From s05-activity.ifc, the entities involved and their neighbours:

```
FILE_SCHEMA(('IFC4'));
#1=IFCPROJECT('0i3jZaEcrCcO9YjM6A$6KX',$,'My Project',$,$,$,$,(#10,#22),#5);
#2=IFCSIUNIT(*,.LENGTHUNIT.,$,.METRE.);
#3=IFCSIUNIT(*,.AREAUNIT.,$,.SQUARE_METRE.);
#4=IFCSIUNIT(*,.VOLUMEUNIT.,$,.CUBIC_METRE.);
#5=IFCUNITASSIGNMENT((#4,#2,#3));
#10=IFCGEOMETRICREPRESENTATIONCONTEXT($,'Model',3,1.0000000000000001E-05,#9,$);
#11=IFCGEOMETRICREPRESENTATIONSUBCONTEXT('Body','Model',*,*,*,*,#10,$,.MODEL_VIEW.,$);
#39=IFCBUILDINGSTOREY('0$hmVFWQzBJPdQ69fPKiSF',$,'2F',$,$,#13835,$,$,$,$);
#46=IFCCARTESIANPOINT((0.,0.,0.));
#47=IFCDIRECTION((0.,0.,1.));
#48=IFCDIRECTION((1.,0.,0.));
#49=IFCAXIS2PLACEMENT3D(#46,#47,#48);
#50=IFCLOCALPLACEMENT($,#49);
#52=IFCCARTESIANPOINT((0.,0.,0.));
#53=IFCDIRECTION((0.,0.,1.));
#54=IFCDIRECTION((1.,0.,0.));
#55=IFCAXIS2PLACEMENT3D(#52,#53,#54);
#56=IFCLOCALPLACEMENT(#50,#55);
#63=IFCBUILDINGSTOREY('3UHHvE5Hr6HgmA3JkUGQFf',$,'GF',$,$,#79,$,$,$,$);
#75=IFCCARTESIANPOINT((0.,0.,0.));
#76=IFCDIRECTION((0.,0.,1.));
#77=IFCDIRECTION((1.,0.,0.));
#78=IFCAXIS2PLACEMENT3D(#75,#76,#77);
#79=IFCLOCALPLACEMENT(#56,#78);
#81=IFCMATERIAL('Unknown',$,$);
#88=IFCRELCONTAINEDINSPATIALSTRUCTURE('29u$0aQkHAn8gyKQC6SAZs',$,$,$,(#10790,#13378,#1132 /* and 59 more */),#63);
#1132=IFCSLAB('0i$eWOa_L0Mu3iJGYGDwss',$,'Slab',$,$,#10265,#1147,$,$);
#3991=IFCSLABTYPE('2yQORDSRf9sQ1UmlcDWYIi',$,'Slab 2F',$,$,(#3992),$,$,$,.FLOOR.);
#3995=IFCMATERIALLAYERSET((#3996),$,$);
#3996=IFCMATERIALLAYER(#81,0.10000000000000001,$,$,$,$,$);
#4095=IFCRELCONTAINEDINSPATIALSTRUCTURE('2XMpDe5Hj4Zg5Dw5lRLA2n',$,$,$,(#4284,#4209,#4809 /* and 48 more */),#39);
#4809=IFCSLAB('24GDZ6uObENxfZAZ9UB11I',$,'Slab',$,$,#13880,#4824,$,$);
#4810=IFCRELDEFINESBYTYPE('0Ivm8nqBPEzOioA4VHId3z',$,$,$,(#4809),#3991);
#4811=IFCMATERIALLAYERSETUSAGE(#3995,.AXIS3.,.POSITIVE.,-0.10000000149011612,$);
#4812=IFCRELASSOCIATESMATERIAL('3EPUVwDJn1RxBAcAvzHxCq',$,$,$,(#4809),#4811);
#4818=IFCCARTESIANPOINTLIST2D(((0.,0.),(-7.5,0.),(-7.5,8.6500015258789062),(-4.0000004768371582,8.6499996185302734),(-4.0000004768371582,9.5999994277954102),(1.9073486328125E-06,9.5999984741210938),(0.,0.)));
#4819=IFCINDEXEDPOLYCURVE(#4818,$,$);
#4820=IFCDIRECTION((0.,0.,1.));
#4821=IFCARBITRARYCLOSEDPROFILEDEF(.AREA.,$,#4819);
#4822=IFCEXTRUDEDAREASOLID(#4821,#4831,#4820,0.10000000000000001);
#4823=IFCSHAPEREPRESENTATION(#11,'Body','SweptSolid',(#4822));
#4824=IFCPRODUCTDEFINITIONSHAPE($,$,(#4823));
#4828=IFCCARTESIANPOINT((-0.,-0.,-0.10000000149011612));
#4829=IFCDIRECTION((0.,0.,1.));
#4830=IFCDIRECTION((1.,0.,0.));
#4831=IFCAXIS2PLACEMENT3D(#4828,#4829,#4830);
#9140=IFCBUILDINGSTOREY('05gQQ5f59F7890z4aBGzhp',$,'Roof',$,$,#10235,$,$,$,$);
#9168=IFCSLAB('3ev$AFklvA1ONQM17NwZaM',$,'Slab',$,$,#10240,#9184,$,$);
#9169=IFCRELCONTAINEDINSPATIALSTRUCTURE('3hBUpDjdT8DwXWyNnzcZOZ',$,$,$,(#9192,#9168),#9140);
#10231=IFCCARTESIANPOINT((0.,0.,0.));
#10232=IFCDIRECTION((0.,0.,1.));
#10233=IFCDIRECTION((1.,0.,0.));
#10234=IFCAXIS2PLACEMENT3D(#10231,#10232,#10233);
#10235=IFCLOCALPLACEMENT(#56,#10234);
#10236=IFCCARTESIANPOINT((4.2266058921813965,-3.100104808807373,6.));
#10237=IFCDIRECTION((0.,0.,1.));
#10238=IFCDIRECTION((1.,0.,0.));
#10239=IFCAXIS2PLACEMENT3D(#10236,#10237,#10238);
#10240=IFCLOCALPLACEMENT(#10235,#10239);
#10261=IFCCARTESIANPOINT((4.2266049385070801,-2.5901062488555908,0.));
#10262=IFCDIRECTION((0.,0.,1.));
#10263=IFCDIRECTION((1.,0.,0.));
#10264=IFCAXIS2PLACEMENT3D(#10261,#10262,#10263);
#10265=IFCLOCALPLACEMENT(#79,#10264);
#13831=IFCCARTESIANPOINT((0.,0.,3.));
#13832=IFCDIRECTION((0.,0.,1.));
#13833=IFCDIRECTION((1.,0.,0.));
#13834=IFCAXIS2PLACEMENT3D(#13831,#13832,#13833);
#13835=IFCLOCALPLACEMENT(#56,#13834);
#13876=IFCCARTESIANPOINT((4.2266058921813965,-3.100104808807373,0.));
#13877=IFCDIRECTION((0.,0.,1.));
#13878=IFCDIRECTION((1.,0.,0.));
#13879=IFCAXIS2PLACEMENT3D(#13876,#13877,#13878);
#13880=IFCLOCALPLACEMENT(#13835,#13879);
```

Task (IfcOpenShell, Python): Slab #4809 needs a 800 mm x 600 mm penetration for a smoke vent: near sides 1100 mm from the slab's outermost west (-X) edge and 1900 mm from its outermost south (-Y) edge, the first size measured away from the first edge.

```python
import numpy as np
import ifcopenshell
import ifcopenshell.api.feature
import ifcopenshell.api.geometry
import ifcopenshell.api.root
import ifcopenshell.geom
import ifcopenshell.util.placement
import ifcopenshell.util.representation
import ifcopenshell.util.shape
import ifcopenshell.util.unit

model = ifcopenshell.open("s05-activity.ifc")
unit_scale = ifcopenshell.util.unit.calculate_unit_scale(model)
settings = ifcopenshell.geom.settings()


def volume(element):
    """Net volume in cubic metres, openings subtracted."""
    shape = ifcopenshell.geom.create_shape(settings, element)
    return ifcopenshell.util.shape.get_volume(shape.geometry)


slab = model.by_guid("24GDZ6uObENxfZAZ9UB11I")
before = volume(slab)

# Extent in the slab's own axes, in metres. The edges named are its -X and -Y sides.
slab_shape = ifcopenshell.geom.create_shape(settings, slab)
vertices = ifcopenshell.util.shape.get_vertices(slab_shape.geometry)
x_min, y_min, bottom = vertices.min(axis=0)
top = vertices[:, 2].max()

opening = ifcopenshell.api.root.create_entity(model, ifc_class="IfcOpeningElement", name="Smoke vent opening", predefined_type="OPENING")
context = ifcopenshell.util.representation.get_context(model, "Model", "Body", "MODEL_VIEW")
width, depth = 0.8, 0.6
outline = [(0.0, 0.0), (width, 0.0), (width, depth), (0.0, depth), (0.0, 0.0)]
# Overshoot both faces by 50 mm so the cut is clean.
shape = ifcopenshell.api.geometry.add_slab_representation(
    model, context=context, depth=top - bottom + 0.1, polyline=outline
)
ifcopenshell.api.geometry.assign_representation(model, product=opening, representation=shape)

matrix = ifcopenshell.util.placement.get_local_placement(slab.ObjectPlacement)
matrix[:, 3] = matrix @ np.append(np.array([x_min + 1.1, y_min + 1.9, bottom - 0.05]) / unit_scale, 1.0)
ifcopenshell.api.geometry.edit_object_placement(model, product=opening, matrix=matrix, is_si=False)
ifcopenshell.api.feature.add_feature(model, feature=opening, element=slab)

after = volume(slab)

print(f"slab volume {before:.3f} -> {after:.3f} m3")

model.write("s05-activity_v2.ifc")
```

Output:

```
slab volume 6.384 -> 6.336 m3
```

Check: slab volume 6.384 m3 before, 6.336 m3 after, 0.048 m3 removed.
